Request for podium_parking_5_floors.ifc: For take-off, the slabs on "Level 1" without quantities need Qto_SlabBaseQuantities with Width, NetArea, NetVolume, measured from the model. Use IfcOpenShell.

First a look at what the model holds.

```python
import ifcopenshell
import ifcopenshell.util.element
import ifcopenshell.util.unit

model = ifcopenshell.open("podium_parking_5_floors.ifc")
print(model.schema)
for unit_type in ("LENGTHUNIT", "AREAUNIT", "VOLUMEUNIT"):
    print(unit_type, ifcopenshell.util.unit.calculate_unit_scale(model, unit_type))
storey = next(s for s in model.by_type("IfcBuildingStorey") if s.Name == "Level 1")
slabs = [e for e in ifcopenshell.util.element.get_decomposition(storey) if e.is_a("IfcSlab")]
for e in sorted(slabs, key=lambda e: e.id()):
    print(e.id(), e.is_a(), e.Name, list(ifcopenshell.util.element.get_psets(e, qtos_only=True)), sep=" | ")
```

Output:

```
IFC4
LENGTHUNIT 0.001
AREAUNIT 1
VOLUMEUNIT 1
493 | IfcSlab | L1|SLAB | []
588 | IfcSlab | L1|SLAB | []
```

```python
import ifcopenshell
import ifcopenshell.api.pset
import ifcopenshell.geom
import ifcopenshell.util.element
import ifcopenshell.util.shape
import ifcopenshell.util.unit

model = ifcopenshell.open("podium_parking_5_floors.ifc")
unit_scale = ifcopenshell.util.unit.calculate_unit_scale(model)
area_scale = ifcopenshell.util.unit.calculate_unit_scale(model, "AREAUNIT")
volume_scale = ifcopenshell.util.unit.calculate_unit_scale(model, "VOLUMEUNIT")
settings = ifcopenshell.geom.settings()

storey = next(s for s in model.by_type("IfcBuildingStorey") if s.Name == "Level 1")
slabs = [e for e in ifcopenshell.util.element.get_decomposition(storey) if e.is_a("IfcSlab")]

for e in sorted(slabs, key=lambda e: e.id()):
    if ifcopenshell.util.element.get_psets(e, qtos_only=True, should_inherit=False):
        continue
    # Geometry comes back in metres, in the element's own axes.
    shape = ifcopenshell.geom.create_shape(settings, e)
    values = {
        "Width": ifcopenshell.util.shape.get_z(shape.geometry) / unit_scale,
        "NetArea": ifcopenshell.util.shape.get_footprint_area(shape.geometry) / area_scale,
        "NetVolume": ifcopenshell.util.shape.get_volume(shape.geometry) / volume_scale,
    }
    qto = ifcopenshell.api.pset.add_qto(model, product=e, name="Qto_SlabBaseQuantities")
    ifcopenshell.api.pset.edit_qto(model, qto=qto, properties=values)
    print(e.id(), {k: round(v, 3) for k, v in values.items()})

model.write("podium_parking_5_floors_edited.ifc")
```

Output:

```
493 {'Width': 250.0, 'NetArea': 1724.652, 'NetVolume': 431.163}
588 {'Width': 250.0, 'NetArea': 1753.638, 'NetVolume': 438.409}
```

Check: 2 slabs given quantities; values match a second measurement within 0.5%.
